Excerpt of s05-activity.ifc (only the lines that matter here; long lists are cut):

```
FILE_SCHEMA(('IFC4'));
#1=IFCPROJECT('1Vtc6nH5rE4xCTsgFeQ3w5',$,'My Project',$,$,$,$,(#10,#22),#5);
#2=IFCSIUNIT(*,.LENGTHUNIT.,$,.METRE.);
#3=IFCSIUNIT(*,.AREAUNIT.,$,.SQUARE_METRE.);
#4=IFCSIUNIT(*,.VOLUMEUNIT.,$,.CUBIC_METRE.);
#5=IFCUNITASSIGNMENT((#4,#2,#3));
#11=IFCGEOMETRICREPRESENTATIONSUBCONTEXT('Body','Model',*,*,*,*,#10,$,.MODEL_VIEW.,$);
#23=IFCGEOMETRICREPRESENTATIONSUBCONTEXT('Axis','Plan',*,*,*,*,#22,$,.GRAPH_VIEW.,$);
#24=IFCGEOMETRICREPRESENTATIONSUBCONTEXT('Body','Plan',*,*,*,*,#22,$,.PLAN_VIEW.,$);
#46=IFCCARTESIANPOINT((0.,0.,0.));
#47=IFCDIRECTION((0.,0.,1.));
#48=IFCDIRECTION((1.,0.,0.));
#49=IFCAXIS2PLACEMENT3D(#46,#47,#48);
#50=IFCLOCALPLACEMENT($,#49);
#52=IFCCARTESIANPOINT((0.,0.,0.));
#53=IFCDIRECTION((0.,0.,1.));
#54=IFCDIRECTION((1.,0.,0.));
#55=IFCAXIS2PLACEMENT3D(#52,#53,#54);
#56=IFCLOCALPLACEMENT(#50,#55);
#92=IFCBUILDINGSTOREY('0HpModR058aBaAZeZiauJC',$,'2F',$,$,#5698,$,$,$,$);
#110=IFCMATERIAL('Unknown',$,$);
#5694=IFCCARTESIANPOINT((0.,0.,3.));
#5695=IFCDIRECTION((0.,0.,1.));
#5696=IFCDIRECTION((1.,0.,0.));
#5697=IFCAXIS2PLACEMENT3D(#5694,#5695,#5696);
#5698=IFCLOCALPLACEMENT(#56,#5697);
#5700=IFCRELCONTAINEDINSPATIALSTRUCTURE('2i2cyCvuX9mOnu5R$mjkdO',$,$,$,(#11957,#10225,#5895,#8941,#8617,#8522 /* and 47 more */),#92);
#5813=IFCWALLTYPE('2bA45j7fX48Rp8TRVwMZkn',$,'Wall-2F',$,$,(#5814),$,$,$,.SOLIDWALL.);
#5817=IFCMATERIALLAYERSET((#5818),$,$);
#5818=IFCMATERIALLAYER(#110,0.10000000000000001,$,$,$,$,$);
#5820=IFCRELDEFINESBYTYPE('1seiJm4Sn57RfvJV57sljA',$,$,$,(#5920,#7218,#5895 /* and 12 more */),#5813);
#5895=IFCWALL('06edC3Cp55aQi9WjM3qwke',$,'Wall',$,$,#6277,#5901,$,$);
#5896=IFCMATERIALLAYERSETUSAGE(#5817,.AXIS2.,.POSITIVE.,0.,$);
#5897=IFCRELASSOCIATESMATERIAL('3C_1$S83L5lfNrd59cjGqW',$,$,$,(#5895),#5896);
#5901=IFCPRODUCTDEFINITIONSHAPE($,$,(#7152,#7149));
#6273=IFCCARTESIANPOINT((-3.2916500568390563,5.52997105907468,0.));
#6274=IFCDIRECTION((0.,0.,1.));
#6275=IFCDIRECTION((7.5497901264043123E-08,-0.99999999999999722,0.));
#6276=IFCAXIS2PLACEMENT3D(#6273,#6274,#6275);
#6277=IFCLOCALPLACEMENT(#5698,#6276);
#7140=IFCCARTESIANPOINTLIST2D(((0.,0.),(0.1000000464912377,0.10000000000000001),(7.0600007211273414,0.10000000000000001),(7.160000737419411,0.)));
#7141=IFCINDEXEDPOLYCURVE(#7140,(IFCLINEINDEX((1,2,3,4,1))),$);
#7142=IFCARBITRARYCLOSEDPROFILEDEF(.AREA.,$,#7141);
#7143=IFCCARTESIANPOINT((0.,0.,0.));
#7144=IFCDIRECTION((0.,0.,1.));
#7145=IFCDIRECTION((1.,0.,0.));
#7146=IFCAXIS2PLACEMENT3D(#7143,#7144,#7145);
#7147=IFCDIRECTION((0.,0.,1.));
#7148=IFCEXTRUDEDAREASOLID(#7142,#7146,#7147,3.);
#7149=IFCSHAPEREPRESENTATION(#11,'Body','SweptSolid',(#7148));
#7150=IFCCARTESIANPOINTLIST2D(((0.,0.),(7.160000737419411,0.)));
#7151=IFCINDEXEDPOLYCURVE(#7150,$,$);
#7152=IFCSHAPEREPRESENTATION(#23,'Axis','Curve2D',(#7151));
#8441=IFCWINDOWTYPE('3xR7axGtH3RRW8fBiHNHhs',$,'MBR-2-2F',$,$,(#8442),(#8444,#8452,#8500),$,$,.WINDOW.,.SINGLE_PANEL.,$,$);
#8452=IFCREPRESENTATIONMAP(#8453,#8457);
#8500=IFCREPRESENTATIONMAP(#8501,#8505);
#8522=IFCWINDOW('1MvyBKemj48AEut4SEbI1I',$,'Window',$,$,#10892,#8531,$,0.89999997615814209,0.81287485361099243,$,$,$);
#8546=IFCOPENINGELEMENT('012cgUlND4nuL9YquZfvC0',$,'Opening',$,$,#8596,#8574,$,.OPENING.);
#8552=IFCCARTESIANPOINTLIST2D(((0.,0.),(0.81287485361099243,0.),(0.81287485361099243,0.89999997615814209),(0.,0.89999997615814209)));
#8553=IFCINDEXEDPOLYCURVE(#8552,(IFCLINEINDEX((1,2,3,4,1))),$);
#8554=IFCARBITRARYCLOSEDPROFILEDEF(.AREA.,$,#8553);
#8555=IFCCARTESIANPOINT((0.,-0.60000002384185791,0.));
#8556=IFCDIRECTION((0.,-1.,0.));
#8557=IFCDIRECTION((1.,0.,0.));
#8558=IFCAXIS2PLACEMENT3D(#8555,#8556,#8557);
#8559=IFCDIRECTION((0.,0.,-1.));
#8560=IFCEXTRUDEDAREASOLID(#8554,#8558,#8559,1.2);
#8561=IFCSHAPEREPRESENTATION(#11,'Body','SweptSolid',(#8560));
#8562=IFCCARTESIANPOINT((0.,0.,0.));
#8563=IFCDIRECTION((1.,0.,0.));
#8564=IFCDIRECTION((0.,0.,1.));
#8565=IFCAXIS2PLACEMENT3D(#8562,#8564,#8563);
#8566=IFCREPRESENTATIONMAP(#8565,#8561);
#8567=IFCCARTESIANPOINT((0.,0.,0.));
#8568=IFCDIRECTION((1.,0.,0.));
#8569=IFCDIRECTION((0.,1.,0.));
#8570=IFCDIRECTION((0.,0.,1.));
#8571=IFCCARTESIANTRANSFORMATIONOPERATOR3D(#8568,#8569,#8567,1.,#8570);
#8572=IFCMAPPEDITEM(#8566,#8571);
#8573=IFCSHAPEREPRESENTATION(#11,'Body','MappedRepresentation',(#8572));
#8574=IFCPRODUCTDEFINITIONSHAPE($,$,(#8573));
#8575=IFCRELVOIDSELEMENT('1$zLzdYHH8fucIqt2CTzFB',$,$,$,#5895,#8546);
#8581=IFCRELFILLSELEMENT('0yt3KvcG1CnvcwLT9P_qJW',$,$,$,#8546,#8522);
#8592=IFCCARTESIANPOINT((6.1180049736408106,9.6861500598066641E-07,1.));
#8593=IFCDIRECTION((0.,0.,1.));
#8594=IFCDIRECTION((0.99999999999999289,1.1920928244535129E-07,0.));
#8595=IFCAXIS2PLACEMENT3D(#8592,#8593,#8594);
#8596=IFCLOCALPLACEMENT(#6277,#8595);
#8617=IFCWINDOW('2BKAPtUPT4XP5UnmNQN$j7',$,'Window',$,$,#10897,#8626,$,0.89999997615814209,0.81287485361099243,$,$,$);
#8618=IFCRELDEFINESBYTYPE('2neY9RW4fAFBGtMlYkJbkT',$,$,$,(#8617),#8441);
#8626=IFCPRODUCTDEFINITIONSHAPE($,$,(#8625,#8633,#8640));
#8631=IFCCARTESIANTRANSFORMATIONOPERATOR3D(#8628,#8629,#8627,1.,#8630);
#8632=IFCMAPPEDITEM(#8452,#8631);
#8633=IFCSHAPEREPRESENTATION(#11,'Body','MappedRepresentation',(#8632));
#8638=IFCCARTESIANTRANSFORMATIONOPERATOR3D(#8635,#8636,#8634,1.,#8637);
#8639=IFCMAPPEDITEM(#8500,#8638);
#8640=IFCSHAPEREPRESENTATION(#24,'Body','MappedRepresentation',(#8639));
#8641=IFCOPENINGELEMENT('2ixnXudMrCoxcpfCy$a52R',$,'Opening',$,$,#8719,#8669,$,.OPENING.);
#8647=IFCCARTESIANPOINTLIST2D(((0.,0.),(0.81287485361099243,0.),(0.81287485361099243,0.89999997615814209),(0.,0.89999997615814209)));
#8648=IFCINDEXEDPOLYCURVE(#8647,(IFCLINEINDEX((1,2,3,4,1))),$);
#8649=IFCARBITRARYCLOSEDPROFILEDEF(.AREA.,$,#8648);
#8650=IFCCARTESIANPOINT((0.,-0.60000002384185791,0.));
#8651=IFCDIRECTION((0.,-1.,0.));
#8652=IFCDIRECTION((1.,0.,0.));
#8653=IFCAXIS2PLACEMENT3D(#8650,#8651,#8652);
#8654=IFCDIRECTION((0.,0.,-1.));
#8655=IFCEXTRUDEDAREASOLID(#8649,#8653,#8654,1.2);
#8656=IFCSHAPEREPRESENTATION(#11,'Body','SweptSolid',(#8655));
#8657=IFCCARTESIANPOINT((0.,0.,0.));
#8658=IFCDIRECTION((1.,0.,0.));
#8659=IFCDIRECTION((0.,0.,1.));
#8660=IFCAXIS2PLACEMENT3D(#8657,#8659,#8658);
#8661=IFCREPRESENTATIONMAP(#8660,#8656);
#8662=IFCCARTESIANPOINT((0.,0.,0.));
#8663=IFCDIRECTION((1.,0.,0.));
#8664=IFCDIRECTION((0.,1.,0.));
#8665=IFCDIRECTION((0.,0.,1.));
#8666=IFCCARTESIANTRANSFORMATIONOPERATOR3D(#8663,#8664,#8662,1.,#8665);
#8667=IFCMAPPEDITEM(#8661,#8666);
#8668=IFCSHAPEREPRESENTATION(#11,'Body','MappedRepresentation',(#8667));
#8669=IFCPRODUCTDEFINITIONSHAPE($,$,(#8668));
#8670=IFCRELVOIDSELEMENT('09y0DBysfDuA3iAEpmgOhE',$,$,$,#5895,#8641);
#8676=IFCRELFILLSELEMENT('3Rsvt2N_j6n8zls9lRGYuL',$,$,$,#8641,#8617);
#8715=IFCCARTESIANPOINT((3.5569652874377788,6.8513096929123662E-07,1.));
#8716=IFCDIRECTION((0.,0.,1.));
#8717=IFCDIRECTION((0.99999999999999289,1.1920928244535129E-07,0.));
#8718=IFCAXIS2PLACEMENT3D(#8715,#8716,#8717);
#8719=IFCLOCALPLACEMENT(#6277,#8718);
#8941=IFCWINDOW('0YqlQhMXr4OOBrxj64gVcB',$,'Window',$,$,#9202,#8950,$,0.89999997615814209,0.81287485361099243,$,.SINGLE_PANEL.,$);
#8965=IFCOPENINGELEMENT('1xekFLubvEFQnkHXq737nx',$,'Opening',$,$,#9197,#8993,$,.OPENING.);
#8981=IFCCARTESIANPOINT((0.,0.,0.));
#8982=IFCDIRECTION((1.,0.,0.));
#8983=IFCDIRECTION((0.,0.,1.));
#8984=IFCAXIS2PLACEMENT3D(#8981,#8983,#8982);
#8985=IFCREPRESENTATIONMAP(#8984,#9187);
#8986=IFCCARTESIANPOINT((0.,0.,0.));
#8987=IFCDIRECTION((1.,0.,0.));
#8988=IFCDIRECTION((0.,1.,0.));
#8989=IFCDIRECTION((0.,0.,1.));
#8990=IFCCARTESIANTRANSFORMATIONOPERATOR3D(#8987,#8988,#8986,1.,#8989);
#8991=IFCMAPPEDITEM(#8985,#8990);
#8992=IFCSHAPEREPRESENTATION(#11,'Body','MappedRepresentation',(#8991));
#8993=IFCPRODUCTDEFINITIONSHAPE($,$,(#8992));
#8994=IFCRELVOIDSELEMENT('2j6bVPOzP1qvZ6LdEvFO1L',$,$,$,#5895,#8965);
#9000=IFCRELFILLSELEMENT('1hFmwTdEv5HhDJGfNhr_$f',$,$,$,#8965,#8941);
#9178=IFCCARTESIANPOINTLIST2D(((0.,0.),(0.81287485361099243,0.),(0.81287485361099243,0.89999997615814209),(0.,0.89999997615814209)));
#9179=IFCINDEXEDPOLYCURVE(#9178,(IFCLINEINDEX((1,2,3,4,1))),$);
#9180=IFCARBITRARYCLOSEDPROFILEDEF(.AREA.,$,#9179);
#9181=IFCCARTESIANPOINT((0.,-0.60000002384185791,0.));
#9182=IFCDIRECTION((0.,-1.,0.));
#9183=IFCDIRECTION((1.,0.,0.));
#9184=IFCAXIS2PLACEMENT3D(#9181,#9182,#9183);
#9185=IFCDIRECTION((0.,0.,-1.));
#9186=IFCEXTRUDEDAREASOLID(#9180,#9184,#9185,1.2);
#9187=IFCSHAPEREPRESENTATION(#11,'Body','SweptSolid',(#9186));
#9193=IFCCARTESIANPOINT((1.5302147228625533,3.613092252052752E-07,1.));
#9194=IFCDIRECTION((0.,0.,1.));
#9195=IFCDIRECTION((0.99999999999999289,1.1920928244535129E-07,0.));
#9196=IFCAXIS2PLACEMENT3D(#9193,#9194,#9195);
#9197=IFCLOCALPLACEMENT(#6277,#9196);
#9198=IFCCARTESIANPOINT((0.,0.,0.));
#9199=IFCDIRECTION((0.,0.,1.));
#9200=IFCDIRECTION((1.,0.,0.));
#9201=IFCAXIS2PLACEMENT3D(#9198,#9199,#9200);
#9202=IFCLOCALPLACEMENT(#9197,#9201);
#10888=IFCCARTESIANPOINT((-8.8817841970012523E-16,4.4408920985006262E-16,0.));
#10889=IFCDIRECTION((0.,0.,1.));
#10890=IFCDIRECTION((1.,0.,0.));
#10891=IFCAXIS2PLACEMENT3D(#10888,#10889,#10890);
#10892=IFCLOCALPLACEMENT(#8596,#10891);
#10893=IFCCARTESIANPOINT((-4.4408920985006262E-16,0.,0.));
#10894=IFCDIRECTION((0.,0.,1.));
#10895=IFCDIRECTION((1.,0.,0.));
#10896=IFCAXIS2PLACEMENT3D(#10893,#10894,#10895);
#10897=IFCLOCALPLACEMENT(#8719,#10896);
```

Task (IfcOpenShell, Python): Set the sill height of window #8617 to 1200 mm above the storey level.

```python
import numpy as np
import ifcopenshell
import ifcopenshell.api.geometry
import ifcopenshell.geom
import ifcopenshell.util.element
import ifcopenshell.util.placement
import ifcopenshell.util.shape
import ifcopenshell.util.unit

model = ifcopenshell.open("s05-activity.ifc")
unit_scale = ifcopenshell.util.unit.calculate_unit_scale(model)

window = model.by_guid("2BKAPtUPT4XP5UnmNQN$j7")
opening = window.FillsVoids[0].RelatingOpeningElement
storey = ifcopenshell.util.element.get_container(window, ifc_class="IfcBuildingStorey")
level = ifcopenshell.util.placement.get_local_placement(storey.ObjectPlacement)[2, 3]

# The opening's origin need not be at the sill, so measure its lowest point.
shape = ifcopenshell.geom.create_shape(ifcopenshell.geom.settings(), opening)
bottom = ifcopenshell.util.shape.get_shape_bottom_elevation(shape, shape.geometry) / unit_scale
dz = level + 1.2 / unit_scale - bottom

shift = np.array([0.0, 0.0, dz])
# The window is placed relative to its opening, so it follows when the opening moves.
matrix = ifcopenshell.util.placement.get_local_placement(opening.ObjectPlacement)
matrix[:3, 3] += shift
ifcopenshell.api.geometry.edit_object_placement(
    model, product=opening, matrix=matrix, is_si=False, should_transform_children=True
)

print(f"moved by {dz * unit_scale:+.3f} m")

model.write("s05-activity_v2.ifc")
```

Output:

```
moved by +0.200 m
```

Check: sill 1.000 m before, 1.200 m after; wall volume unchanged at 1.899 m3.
